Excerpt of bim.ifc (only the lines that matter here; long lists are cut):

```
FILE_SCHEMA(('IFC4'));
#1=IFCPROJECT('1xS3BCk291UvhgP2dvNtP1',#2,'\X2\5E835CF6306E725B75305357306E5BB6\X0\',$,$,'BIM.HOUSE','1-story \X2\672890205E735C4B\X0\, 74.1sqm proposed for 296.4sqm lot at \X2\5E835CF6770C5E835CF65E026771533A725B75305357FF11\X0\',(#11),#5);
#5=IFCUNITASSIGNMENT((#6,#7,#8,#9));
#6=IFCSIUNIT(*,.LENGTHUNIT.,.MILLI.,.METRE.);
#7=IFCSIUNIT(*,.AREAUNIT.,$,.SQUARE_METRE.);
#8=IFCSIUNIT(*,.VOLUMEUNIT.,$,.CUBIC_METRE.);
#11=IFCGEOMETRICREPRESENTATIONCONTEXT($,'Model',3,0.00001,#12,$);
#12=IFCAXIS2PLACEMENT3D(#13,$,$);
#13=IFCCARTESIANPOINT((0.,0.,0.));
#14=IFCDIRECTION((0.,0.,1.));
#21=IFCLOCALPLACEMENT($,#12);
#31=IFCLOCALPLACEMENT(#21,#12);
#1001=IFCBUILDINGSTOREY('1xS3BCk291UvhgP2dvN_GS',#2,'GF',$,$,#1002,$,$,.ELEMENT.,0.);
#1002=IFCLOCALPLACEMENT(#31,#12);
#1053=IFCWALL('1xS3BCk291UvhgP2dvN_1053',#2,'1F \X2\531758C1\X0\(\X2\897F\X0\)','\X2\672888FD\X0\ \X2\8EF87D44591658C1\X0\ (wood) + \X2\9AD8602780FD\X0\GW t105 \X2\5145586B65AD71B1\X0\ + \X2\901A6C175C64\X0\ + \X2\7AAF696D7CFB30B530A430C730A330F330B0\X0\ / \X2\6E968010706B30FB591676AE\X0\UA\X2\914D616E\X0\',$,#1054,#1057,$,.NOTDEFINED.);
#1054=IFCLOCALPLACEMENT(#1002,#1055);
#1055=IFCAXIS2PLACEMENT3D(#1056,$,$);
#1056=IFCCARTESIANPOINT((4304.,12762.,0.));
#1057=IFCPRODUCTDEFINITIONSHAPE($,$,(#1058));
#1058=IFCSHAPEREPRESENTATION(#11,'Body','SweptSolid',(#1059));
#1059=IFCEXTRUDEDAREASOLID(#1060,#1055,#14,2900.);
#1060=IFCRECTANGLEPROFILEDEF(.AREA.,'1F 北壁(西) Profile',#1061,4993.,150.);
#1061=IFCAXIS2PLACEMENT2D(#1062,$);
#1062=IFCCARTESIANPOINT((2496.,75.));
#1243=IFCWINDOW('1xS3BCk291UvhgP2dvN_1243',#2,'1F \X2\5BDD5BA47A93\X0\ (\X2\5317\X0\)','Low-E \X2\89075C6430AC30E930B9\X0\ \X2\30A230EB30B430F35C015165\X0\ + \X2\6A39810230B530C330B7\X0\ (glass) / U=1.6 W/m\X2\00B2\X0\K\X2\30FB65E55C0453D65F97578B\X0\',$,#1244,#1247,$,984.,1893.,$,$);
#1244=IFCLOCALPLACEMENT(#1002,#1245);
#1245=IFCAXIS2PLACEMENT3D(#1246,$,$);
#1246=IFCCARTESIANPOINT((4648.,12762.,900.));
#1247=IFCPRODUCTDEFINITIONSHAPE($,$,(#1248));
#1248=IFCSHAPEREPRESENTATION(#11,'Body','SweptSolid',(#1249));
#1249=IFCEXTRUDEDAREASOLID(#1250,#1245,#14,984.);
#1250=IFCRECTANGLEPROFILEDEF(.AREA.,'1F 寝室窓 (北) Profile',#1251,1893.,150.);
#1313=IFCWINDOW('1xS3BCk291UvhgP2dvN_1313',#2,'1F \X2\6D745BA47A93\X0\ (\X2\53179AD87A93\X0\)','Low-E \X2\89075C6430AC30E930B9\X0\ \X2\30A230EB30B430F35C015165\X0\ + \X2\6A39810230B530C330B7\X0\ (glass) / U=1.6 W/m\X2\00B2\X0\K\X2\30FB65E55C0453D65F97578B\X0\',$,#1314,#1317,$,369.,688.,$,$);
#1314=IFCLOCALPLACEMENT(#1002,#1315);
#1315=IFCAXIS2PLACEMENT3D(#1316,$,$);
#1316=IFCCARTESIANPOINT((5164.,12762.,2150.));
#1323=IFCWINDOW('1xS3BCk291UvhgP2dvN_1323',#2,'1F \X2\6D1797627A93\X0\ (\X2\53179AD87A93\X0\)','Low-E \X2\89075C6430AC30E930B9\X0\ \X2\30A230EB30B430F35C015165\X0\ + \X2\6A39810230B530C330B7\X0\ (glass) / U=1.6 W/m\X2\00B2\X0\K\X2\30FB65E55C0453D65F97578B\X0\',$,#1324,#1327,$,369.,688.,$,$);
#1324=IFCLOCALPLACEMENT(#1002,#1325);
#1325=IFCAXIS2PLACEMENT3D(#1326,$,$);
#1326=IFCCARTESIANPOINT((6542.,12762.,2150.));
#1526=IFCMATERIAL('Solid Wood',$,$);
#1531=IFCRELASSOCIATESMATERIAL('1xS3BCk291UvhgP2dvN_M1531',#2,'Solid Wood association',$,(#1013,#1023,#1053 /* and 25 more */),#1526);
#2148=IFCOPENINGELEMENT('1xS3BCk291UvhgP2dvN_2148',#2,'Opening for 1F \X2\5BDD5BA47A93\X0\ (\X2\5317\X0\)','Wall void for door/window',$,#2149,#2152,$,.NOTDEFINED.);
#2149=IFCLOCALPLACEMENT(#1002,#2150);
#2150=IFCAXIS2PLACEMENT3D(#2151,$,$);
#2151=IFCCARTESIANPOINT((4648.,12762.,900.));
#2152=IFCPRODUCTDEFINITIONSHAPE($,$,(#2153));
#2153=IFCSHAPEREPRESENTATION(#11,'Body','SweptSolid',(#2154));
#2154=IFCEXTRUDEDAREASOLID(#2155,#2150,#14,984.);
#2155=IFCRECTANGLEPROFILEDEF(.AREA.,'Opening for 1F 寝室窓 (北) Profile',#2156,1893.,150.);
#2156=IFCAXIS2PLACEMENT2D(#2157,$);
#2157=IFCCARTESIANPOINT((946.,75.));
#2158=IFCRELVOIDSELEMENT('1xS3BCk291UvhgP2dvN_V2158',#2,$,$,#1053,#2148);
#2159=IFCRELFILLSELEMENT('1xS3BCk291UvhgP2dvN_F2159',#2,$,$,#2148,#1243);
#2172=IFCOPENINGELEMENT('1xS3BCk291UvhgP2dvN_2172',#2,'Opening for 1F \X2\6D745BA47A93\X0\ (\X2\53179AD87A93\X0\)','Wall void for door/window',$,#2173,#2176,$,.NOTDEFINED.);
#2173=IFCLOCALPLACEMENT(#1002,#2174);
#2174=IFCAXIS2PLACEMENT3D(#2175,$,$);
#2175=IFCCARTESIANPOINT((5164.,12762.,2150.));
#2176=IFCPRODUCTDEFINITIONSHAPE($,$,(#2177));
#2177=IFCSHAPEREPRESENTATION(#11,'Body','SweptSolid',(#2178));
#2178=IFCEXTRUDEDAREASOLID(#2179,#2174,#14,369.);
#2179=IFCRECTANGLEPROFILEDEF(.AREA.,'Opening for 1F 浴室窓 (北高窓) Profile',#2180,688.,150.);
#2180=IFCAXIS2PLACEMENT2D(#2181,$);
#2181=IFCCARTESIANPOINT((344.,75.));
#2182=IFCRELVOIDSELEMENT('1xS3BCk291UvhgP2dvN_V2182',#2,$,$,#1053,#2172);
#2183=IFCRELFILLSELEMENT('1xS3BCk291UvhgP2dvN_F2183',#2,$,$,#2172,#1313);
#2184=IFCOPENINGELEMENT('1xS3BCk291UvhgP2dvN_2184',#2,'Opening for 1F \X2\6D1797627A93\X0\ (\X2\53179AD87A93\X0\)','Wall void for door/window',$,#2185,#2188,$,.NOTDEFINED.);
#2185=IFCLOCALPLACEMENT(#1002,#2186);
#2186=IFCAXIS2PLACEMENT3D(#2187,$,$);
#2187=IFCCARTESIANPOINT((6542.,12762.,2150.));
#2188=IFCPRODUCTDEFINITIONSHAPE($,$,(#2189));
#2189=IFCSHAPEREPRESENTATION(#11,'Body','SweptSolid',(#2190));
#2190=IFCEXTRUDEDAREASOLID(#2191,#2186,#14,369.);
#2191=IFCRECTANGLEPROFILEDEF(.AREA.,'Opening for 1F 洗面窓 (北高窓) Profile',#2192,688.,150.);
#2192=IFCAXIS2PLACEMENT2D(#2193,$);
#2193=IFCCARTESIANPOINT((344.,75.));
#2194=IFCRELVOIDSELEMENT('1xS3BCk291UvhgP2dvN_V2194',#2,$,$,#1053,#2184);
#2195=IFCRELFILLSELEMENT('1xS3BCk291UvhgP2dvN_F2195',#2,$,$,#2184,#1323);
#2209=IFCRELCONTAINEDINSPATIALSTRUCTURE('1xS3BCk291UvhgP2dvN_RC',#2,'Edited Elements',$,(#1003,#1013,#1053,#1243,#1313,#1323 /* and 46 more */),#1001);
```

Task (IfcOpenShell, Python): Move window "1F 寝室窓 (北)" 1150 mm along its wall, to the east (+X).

```python
import ifcopenshell
import ifcopenshell.api.geometry
import ifcopenshell.util.placement
import ifcopenshell.util.unit

model = ifcopenshell.open("bim.ifc")
unit_scale = ifcopenshell.util.unit.calculate_unit_scale(model)

window = model.by_guid("1xS3BCk291UvhgP2dvN_1243")
opening = window.FillsVoids[0].RelatingOpeningElement
wall = opening.VoidsElements[0].RelatingBuildingElement

wall_matrix = ifcopenshell.util.placement.get_local_placement(wall.ObjectPlacement)
shift = wall_matrix[:3, 0] * 1.15 / unit_scale
before = ifcopenshell.util.placement.get_local_placement(window.ObjectPlacement)[:3, 3].copy()

# The window is not placed relative to its opening, so move both.
for product in (opening, window):
    matrix = ifcopenshell.util.placement.get_local_placement(product.ObjectPlacement)
    matrix[:3, 3] += shift
    ifcopenshell.api.geometry.edit_object_placement(model, product=product, matrix=matrix, is_si=False)

after = ifcopenshell.util.placement.get_local_placement(window.ObjectPlacement)[:3, 3]
print("window moved by", (after - before).round(3) + 0.0)

model.write("bim_v2.ifc")
```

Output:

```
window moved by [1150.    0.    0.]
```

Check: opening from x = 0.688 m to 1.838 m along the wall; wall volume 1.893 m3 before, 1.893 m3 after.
